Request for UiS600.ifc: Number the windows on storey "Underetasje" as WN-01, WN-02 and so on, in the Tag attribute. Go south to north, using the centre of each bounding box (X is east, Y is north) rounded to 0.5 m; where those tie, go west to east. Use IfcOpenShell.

First a look at what the model holds.

```python
import ifcopenshell
import ifcopenshell.util.element
import ifcopenshell.util.placement

model = ifcopenshell.open("UiS600.ifc")
print(model.schema)
storey = next(s for s in model.by_type("IfcBuildingStorey") if s.Name == "Underetasje")
windows = [e for e in ifcopenshell.util.element.get_decomposition(storey) if e.is_a("IfcWindow")]
for e in sorted(windows, key=lambda e: e.id()):
    origin = ifcopenshell.util.placement.get_local_placement(e.ObjectPlacement)[:3, 3]
    print(e.id(), e.Tag, e.Name, origin.round(2) + 0.0, sep=" | ")
```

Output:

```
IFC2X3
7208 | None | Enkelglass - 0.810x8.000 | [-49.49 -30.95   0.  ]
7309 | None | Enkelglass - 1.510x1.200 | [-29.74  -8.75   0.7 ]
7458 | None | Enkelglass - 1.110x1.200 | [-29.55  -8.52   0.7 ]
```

```python
import ifcopenshell
import ifcopenshell.geom
import ifcopenshell.util.element
import ifcopenshell.util.shape

model = ifcopenshell.open("UiS600.ifc")
settings = ifcopenshell.geom.settings()
settings.set("use-world-coords", True)


def centre(element):
    shape = ifcopenshell.geom.create_shape(settings, element)
    return ifcopenshell.util.shape.get_bbox_centroid(shape.geometry)


storey = next(s for s in model.by_type("IfcBuildingStorey") if s.Name == "Underetasje")
windows = [e for e in ifcopenshell.util.element.get_decomposition(storey) if e.is_a("IfcWindow")]

# Insertion points can sit at a corner or the storey origin, so sort by the geometry (in metres).
centres = {e: centre(e) for e in windows}
windows.sort(key=lambda e: (round(centres[e][1] / 0.5), centres[e][0]))

for i, e in enumerate(windows, start=1):
    number = f"WN-{i:02d}"
    e.Tag = number
    print(e.id(), number)

model.write("UiS600-out.ifc")
```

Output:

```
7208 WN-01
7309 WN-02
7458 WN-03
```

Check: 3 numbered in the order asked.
